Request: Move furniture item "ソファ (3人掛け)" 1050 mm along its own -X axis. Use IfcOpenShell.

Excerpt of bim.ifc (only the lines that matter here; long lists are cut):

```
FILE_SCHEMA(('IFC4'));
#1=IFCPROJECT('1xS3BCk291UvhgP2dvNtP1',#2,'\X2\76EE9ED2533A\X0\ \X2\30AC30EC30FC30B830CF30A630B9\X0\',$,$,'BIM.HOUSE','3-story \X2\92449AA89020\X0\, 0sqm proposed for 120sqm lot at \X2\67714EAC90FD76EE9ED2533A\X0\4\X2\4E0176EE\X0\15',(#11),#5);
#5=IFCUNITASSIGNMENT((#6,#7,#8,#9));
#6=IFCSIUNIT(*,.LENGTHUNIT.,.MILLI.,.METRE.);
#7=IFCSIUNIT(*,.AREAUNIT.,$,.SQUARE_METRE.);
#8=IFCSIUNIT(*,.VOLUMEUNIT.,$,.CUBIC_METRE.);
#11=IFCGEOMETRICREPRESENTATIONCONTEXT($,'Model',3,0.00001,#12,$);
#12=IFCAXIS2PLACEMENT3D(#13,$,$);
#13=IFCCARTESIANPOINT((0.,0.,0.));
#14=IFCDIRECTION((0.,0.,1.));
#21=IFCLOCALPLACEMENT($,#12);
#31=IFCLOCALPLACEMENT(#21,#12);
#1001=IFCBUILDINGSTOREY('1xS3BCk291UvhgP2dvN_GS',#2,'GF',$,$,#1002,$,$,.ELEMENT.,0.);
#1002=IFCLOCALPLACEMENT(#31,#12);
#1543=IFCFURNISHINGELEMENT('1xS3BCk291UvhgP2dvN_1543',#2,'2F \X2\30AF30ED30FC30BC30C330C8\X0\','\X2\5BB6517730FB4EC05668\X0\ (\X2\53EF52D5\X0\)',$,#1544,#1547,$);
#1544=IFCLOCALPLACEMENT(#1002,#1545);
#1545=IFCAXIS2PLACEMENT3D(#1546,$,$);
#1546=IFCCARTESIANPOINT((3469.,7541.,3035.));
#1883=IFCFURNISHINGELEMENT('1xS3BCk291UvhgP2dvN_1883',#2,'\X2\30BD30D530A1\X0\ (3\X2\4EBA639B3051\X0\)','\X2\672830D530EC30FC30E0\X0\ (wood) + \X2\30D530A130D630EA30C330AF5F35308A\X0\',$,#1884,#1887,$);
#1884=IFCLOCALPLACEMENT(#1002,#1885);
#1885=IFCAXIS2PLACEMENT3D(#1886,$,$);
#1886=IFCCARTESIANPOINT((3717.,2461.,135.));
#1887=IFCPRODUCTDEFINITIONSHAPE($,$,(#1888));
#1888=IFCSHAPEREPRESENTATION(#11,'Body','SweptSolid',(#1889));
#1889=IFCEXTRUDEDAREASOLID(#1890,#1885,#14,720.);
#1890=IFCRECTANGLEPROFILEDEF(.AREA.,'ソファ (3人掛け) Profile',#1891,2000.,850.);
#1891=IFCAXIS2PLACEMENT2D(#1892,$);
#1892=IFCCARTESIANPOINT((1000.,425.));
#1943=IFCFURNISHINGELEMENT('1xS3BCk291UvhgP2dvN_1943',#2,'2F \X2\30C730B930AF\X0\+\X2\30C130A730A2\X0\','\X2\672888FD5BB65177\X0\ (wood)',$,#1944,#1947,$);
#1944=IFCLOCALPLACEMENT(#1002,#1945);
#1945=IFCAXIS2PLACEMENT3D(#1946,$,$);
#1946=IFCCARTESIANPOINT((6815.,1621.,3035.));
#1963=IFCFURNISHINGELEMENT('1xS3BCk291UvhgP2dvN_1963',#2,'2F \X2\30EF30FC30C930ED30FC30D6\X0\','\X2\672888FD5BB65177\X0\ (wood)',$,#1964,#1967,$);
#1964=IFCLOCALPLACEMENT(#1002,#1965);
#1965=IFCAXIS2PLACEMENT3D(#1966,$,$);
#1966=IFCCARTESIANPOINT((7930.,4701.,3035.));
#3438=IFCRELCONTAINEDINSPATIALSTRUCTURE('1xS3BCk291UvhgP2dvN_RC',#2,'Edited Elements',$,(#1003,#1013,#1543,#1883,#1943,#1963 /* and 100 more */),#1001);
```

```python
import ifcopenshell
import ifcopenshell.api.geometry
import ifcopenshell.util.placement

model = ifcopenshell.open("bim.ifc")

item = model.by_guid("1xS3BCk291UvhgP2dvN_1883")
matrix = ifcopenshell.util.placement.get_local_placement(item.ObjectPlacement)
matrix[:3, 3] -= matrix[:3, 0] * 1050.0
ifcopenshell.api.geometry.edit_object_placement(model, product=item, matrix=matrix, is_si=False)

print(ifcopenshell.util.placement.get_local_placement(item.ObjectPlacement).round(3) + 0.0)

model.write("bim_rev.ifc")
```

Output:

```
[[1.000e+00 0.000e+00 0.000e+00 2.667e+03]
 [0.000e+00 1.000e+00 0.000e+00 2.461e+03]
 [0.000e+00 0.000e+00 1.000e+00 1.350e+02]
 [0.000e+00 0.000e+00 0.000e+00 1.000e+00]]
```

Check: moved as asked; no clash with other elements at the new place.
